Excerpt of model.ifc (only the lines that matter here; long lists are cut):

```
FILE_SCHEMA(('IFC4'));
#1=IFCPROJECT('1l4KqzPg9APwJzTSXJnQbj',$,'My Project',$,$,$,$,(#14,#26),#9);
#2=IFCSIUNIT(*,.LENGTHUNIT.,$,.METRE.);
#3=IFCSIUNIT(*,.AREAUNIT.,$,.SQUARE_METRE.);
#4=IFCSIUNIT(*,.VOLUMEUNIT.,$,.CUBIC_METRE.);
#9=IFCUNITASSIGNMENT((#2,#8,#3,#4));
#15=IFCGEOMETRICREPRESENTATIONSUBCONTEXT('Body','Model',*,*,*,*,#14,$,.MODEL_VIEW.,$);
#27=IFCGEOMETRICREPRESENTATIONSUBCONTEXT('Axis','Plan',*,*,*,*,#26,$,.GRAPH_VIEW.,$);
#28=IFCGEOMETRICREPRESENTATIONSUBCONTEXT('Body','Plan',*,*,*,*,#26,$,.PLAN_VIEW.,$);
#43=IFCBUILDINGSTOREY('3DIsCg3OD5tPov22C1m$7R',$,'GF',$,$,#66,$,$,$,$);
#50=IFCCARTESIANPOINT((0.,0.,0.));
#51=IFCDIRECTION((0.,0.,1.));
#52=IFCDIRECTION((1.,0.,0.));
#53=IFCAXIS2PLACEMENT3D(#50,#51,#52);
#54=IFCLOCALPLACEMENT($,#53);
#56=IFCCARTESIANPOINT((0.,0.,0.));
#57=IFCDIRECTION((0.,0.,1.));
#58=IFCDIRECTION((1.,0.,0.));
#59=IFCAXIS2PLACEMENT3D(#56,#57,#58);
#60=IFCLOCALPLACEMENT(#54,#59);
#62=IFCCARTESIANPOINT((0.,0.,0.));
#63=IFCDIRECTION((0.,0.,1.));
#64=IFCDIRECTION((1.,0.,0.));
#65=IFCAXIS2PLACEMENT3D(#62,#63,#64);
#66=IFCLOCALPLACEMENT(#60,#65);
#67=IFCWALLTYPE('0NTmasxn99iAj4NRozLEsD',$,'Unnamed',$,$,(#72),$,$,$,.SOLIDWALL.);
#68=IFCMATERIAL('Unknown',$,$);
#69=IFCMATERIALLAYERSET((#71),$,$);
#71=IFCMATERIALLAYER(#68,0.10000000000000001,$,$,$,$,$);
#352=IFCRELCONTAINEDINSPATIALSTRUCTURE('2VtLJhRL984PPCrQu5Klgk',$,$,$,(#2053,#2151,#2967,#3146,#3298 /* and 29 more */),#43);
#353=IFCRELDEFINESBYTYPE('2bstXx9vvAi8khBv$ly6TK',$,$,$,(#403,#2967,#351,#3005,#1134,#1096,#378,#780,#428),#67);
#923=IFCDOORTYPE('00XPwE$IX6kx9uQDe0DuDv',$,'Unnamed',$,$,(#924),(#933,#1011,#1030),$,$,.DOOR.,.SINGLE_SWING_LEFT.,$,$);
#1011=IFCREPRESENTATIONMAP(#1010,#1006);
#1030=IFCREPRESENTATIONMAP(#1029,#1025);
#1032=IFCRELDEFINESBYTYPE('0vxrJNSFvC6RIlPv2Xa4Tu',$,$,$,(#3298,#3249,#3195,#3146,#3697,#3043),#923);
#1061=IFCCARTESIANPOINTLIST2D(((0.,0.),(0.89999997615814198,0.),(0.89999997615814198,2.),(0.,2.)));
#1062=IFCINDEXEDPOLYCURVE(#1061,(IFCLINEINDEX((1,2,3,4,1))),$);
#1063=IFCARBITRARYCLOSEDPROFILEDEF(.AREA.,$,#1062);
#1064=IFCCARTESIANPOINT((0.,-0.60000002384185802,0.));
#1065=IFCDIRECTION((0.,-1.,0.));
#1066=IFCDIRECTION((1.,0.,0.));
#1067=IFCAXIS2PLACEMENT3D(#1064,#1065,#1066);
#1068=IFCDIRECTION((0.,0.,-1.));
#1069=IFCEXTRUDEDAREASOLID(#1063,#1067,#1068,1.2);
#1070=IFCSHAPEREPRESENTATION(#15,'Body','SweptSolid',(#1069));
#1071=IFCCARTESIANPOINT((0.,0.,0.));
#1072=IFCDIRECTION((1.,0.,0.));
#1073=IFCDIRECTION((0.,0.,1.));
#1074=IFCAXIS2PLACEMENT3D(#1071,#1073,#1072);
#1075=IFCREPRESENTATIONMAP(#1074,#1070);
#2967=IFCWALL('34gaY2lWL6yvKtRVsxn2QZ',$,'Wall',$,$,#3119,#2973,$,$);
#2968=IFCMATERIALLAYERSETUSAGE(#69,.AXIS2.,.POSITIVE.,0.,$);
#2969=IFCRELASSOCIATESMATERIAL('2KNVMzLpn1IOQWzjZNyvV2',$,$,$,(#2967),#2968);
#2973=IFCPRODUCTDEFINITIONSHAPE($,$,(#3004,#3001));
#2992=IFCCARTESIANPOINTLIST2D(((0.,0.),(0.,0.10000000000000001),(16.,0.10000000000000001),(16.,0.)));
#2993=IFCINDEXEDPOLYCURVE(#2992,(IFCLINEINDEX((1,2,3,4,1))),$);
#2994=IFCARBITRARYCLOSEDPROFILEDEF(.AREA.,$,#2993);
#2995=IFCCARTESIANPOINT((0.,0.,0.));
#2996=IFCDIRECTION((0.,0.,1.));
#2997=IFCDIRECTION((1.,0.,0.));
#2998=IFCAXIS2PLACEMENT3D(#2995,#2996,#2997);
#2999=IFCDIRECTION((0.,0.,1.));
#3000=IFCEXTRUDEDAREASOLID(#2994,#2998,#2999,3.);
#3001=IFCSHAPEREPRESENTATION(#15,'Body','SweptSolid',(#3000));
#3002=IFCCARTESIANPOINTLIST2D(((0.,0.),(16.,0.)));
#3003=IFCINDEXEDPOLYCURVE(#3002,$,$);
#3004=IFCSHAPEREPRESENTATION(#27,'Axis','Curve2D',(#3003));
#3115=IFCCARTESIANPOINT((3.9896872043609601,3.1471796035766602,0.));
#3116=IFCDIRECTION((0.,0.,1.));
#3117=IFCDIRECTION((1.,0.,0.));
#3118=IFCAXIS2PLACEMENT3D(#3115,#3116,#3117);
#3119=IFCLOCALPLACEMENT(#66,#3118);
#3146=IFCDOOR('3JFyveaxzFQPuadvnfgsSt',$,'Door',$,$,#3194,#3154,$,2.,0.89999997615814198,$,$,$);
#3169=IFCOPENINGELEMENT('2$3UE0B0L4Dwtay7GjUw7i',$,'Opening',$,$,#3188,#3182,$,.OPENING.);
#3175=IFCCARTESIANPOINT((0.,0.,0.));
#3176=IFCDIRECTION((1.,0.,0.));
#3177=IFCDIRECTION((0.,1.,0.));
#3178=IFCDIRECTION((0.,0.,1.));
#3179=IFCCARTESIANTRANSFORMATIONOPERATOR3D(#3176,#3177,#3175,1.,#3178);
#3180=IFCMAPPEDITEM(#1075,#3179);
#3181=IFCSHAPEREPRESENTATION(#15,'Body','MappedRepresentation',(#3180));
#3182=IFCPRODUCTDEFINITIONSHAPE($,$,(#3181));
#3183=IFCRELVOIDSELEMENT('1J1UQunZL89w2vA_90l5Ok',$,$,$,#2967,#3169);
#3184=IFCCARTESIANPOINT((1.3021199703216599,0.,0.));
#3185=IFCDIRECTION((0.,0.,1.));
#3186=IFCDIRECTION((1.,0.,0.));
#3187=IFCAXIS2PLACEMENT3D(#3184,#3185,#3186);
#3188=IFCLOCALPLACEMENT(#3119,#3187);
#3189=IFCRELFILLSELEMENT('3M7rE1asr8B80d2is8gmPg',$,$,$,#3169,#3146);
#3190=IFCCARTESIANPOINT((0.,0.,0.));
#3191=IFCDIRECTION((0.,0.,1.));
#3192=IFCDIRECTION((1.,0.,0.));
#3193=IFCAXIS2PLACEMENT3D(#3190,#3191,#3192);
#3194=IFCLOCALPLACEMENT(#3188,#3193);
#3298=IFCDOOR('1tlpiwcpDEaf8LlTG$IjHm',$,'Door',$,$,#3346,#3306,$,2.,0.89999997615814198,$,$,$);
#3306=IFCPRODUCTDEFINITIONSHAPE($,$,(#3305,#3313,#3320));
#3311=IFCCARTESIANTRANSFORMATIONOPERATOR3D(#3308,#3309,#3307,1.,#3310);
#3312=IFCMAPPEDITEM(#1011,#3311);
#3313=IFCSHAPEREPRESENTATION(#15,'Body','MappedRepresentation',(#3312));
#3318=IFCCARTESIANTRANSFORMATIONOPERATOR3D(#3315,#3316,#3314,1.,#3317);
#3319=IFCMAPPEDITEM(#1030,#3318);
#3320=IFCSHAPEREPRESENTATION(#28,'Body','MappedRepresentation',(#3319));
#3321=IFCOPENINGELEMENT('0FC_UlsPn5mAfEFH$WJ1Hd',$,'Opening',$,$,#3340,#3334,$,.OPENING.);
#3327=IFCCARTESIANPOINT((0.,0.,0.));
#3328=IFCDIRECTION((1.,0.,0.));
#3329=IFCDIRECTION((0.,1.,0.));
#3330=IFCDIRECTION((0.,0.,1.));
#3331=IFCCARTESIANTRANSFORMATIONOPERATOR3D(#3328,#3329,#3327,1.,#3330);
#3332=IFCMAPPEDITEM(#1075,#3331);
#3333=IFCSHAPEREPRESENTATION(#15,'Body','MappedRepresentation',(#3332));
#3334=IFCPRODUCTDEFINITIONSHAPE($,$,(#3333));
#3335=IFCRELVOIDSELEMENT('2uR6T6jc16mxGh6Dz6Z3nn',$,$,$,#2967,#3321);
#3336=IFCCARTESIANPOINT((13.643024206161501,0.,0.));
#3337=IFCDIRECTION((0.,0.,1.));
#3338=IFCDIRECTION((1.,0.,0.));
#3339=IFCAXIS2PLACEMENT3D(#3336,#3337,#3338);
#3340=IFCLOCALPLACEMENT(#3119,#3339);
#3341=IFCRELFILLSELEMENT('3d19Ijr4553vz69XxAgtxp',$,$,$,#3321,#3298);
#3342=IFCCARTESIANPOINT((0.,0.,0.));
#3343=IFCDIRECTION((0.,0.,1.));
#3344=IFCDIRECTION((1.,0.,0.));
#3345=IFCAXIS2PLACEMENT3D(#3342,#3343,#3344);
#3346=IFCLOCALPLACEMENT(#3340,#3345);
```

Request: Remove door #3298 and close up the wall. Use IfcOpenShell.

```python
import ifcopenshell
import ifcopenshell.api.feature
import ifcopenshell.api.root
import ifcopenshell.geom
import ifcopenshell.util.shape

model = ifcopenshell.open("model.ifc")
settings = ifcopenshell.geom.settings()


def volume(element):
    """Net volume in cubic metres, openings subtracted."""
    shape = ifcopenshell.geom.create_shape(settings, element)
    return ifcopenshell.util.shape.get_volume(shape.geometry)


door = model.by_guid("1tlpiwcpDEaf8LlTG$IjHm")
opening = door.FillsVoids[0].RelatingOpeningElement
wall = opening.VoidsElements[0].RelatingBuildingElement
before = volume(wall)

ifcopenshell.api.root.remove_product(model, product=door)
ifcopenshell.api.feature.remove_feature(model, feature=opening)

after = volume(wall)

print(f"wall volume {before:.3f} -> {after:.3f} m3")

model.write("model_updated.ifc")
```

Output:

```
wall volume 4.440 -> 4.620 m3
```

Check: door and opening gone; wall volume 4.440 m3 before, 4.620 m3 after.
